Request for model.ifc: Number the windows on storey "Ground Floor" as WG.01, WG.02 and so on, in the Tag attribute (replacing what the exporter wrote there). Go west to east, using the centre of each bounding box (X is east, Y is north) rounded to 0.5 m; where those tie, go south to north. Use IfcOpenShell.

First a look at what the model holds.

```python
import ifcopenshell
import ifcopenshell.util.element
import ifcopenshell.util.placement

model = ifcopenshell.open("model.ifc")
print(model.schema)
storey = next(s for s in model.by_type("IfcBuildingStorey") if s.Name == "Ground Floor")
windows = [e for e in ifcopenshell.util.element.get_decomposition(storey) if e.is_a("IfcWindow")]
for e in sorted(windows, key=lambda e: e.id()):
    origin = ifcopenshell.util.placement.get_local_placement(e.ObjectPlacement)[:3, 3]
    print(e.id(), e.Tag, e.Name, origin.round(2) + 0.0, sep=" | ")
```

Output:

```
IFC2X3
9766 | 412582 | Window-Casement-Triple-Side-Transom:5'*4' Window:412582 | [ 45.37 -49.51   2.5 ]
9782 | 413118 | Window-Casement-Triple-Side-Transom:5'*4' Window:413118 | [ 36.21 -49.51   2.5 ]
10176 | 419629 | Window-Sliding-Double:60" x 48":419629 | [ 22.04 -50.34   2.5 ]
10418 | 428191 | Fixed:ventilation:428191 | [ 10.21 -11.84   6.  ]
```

```python
import ifcopenshell
import ifcopenshell.geom
import ifcopenshell.util.element
import ifcopenshell.util.shape

model = ifcopenshell.open("model.ifc")
settings = ifcopenshell.geom.settings()
settings.set("use-world-coords", True)


def centre(element):
    shape = ifcopenshell.geom.create_shape(settings, element)
    return ifcopenshell.util.shape.get_bbox_centroid(shape.geometry)


storey = next(s for s in model.by_type("IfcBuildingStorey") if s.Name == "Ground Floor")
windows = [e for e in ifcopenshell.util.element.get_decomposition(storey) if e.is_a("IfcWindow")]

# Insertion points can sit at a corner or the storey origin, so sort by the geometry (in metres).
centres = {e: centre(e) for e in windows}
windows.sort(key=lambda e: (round(centres[e][0] / 0.5), centres[e][1]))

for i, e in enumerate(windows, start=1):
    number = f"WG.{i:02d}"
    e.Tag = number
    print(e.id(), number)

model.write("model_edited.ifc")
```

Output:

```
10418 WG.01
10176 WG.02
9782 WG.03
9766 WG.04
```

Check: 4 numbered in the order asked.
